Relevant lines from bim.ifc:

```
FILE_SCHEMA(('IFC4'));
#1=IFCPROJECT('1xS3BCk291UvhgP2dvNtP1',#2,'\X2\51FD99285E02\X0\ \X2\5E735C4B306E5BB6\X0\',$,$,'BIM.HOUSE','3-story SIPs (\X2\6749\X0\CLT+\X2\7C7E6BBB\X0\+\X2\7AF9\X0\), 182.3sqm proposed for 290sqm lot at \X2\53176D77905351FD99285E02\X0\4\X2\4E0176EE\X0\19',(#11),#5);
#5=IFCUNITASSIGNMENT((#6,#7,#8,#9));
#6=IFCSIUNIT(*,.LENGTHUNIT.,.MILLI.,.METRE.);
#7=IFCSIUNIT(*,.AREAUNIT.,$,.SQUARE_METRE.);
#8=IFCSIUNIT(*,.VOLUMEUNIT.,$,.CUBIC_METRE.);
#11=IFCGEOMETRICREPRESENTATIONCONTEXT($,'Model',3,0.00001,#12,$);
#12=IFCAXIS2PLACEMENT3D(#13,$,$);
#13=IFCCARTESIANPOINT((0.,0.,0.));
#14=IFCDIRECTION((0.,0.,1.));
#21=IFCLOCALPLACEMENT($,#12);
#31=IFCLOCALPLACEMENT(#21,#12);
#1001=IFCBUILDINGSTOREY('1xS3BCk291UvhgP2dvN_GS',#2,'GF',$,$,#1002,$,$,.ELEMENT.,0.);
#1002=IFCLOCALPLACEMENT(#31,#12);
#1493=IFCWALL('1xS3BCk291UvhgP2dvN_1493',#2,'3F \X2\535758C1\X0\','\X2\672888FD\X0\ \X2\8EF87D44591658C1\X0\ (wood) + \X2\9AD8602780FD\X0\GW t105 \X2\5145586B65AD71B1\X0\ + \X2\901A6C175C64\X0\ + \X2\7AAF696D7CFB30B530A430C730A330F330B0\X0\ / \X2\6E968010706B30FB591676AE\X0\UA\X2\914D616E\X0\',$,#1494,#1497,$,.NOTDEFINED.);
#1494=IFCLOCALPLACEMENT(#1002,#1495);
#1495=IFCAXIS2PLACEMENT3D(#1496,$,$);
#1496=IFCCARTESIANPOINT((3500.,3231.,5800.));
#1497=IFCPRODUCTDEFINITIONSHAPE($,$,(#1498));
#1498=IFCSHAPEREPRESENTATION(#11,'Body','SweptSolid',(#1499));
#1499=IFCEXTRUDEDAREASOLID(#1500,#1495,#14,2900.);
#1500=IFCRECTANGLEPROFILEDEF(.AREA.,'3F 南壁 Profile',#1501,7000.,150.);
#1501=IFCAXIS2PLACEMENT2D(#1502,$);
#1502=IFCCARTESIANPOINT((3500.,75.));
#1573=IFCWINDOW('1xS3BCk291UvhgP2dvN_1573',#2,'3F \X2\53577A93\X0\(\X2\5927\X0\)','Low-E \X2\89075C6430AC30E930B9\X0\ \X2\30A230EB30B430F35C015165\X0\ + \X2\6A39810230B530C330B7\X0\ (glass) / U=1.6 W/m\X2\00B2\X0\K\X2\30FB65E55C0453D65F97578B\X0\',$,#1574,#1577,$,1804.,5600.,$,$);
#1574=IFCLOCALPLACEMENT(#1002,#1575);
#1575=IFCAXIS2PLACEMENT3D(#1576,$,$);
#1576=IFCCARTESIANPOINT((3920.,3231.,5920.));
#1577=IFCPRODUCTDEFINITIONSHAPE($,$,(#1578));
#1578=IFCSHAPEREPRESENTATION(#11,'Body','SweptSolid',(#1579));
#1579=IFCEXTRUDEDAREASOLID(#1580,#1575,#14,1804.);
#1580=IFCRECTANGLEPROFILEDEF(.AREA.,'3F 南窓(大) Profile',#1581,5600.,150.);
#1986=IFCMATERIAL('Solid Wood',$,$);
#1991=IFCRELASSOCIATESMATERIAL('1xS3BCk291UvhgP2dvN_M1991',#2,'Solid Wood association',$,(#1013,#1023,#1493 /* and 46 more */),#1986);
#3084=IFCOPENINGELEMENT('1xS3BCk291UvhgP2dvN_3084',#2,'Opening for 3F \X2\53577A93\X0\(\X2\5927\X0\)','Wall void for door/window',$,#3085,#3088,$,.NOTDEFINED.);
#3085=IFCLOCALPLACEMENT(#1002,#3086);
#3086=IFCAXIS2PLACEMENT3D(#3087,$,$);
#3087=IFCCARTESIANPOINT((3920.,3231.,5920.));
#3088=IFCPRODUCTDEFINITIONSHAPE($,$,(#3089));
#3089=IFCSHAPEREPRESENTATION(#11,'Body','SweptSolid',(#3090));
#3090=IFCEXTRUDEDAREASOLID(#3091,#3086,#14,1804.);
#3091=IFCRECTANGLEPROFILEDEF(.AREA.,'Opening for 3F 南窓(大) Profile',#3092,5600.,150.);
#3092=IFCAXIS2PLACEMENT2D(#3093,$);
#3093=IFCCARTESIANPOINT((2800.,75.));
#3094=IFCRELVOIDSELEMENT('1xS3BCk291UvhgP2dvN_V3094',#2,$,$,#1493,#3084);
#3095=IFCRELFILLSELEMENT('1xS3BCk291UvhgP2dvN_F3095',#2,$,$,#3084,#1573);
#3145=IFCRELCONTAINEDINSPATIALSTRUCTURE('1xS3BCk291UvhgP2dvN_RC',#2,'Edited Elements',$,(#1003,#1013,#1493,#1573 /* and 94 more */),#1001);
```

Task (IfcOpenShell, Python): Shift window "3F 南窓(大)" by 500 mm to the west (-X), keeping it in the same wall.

```python
import ifcopenshell
import ifcopenshell.api.geometry
import ifcopenshell.util.placement
import ifcopenshell.util.unit

model = ifcopenshell.open("bim.ifc")
unit_scale = ifcopenshell.util.unit.calculate_unit_scale(model)

window = model.by_guid("1xS3BCk291UvhgP2dvN_1573")
opening = window.FillsVoids[0].RelatingOpeningElement
wall = opening.VoidsElements[0].RelatingBuildingElement

wall_matrix = ifcopenshell.util.placement.get_local_placement(wall.ObjectPlacement)
shift = wall_matrix[:3, 0] * -0.5 / unit_scale
before = ifcopenshell.util.placement.get_local_placement(window.ObjectPlacement)[:3, 3].copy()

# The window is not placed relative to its opening, so move both.
for product in (opening, window):
    matrix = ifcopenshell.util.placement.get_local_placement(product.ObjectPlacement)
    matrix[:3, 3] += shift
    ifcopenshell.api.geometry.edit_object_placement(model, product=product, matrix=matrix, is_si=False)

after = ifcopenshell.util.placement.get_local_placement(window.ObjectPlacement)[:3, 3]
print("window moved by", (after - before).round(3) + 0.0)

model.write("bim_v2.ifc")
```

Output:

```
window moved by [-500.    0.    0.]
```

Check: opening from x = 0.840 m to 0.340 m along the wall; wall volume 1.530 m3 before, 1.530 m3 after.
